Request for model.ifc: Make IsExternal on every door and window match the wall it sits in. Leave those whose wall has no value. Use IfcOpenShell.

First a look at what the model holds.

```python
import ifcopenshell
import ifcopenshell.util.element

model = ifcopenshell.open("model.ifc")
print(model.schema)
seen = {}
for e in model.by_type("IfcDoor") + model.by_type("IfcWindow"):
    if not e.FillsVoids:
        continue
    host = e.FillsVoids[0].RelatingOpeningElement.VoidsElements[0].RelatingBuildingElement
    own = ifcopenshell.util.element.get_pset(e, f"Pset_{e.is_a()[3:].removesuffix('StandardCase')}Common", "IsExternal")
    wall = ifcopenshell.util.element.get_pset(host, "Pset_WallCommon", "IsExternal")
    seen[e.is_a(), own, wall] = seen.get((e.is_a(), own, wall), 0) + 1
for (cls, own, wall), count in sorted(seen.items(), key=str):
    print(count, cls, "IsExternal:", own, "| host wall:", wall)
```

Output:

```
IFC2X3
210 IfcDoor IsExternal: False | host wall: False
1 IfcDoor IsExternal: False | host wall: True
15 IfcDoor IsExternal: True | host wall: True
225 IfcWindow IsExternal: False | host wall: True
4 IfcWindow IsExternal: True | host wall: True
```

```python
import ifcopenshell
import ifcopenshell.api.pset
import ifcopenshell.util.element

model = ifcopenshell.open("model.ifc")

count = 0
for ifc_class, pset_name in (("IfcDoor", "Pset_DoorCommon"), ("IfcWindow", "Pset_WindowCommon")):
    for e in model.by_type(ifc_class):
        if not e.FillsVoids:
            continue
        host = e.FillsVoids[0].RelatingOpeningElement.VoidsElements[0].RelatingBuildingElement
        external = ifcopenshell.util.element.get_pset(host, "Pset_WallCommon", "IsExternal")
        if external is None or ifcopenshell.util.element.get_pset(e, pset_name, "IsExternal") == external:
            continue
        pset = ifcopenshell.api.pset.add_pset(model, product=e, name=pset_name)
        ifcopenshell.api.pset.edit_pset(model, pset=pset, properties={"IsExternal": external})
        count += 1

print(count, "updated")

model.write("model_rev.ifc")
```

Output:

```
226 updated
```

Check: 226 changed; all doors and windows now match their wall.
